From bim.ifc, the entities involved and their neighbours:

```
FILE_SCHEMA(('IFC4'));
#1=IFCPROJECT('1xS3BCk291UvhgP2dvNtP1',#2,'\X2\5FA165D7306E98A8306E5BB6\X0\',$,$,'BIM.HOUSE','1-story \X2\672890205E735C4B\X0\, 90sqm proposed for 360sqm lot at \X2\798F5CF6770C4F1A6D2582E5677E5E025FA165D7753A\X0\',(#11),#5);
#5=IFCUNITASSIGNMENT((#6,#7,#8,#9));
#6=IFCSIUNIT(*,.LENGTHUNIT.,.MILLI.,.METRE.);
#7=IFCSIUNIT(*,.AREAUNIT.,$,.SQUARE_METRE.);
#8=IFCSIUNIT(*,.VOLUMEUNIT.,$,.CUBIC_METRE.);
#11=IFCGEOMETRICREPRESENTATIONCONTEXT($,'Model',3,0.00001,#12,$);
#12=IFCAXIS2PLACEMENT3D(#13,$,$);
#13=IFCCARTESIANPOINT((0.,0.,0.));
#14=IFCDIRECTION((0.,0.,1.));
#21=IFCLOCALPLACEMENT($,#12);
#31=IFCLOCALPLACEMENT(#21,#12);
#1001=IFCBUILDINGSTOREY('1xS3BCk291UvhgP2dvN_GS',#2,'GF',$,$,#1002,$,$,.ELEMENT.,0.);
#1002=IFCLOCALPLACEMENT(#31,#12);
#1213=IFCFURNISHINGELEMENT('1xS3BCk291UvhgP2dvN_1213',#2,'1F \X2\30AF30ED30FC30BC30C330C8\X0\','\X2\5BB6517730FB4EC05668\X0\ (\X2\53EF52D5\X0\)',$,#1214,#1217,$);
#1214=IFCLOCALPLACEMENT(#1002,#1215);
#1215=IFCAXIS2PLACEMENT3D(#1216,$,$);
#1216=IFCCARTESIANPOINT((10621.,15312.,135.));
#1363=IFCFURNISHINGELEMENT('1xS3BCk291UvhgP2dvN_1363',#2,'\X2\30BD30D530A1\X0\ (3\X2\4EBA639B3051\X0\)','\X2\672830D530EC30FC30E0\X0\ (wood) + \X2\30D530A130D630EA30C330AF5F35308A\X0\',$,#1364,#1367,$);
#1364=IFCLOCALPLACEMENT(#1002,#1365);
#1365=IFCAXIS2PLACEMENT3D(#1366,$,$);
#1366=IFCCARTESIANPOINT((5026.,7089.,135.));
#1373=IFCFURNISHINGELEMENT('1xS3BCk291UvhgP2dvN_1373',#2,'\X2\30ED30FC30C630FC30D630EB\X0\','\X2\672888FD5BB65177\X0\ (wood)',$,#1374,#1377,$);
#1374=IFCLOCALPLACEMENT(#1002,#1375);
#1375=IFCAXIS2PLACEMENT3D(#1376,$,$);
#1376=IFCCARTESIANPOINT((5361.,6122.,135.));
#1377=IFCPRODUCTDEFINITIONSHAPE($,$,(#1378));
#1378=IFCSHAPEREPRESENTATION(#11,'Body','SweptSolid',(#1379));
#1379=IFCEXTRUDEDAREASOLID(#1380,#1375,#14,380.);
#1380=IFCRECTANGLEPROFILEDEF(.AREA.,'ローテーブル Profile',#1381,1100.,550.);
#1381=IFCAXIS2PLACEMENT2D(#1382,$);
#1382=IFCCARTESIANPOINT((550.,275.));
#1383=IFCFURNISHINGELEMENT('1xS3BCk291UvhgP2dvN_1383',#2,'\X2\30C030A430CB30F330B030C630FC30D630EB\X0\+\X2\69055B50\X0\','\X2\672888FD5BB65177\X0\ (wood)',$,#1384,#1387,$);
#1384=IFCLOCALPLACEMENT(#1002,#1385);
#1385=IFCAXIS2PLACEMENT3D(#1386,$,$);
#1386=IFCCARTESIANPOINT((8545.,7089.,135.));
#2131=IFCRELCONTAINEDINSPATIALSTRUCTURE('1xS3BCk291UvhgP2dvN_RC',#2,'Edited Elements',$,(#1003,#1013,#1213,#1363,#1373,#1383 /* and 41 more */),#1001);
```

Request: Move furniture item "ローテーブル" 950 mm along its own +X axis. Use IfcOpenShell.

```python
import ifcopenshell
import ifcopenshell.api.geometry
import ifcopenshell.util.placement

model = ifcopenshell.open("bim.ifc")

item = model.by_guid("1xS3BCk291UvhgP2dvN_1373")
matrix = ifcopenshell.util.placement.get_local_placement(item.ObjectPlacement)
matrix[:3, 3] += matrix[:3, 0] * 950.0
ifcopenshell.api.geometry.edit_object_placement(model, product=item, matrix=matrix, is_si=False)

print(ifcopenshell.util.placement.get_local_placement(item.ObjectPlacement).round(3) + 0.0)

model.write("bim_updated.ifc")
```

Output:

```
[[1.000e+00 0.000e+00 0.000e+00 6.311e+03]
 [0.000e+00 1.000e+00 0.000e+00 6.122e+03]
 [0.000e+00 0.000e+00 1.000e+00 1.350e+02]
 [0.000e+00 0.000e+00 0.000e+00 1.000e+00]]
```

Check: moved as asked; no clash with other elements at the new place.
